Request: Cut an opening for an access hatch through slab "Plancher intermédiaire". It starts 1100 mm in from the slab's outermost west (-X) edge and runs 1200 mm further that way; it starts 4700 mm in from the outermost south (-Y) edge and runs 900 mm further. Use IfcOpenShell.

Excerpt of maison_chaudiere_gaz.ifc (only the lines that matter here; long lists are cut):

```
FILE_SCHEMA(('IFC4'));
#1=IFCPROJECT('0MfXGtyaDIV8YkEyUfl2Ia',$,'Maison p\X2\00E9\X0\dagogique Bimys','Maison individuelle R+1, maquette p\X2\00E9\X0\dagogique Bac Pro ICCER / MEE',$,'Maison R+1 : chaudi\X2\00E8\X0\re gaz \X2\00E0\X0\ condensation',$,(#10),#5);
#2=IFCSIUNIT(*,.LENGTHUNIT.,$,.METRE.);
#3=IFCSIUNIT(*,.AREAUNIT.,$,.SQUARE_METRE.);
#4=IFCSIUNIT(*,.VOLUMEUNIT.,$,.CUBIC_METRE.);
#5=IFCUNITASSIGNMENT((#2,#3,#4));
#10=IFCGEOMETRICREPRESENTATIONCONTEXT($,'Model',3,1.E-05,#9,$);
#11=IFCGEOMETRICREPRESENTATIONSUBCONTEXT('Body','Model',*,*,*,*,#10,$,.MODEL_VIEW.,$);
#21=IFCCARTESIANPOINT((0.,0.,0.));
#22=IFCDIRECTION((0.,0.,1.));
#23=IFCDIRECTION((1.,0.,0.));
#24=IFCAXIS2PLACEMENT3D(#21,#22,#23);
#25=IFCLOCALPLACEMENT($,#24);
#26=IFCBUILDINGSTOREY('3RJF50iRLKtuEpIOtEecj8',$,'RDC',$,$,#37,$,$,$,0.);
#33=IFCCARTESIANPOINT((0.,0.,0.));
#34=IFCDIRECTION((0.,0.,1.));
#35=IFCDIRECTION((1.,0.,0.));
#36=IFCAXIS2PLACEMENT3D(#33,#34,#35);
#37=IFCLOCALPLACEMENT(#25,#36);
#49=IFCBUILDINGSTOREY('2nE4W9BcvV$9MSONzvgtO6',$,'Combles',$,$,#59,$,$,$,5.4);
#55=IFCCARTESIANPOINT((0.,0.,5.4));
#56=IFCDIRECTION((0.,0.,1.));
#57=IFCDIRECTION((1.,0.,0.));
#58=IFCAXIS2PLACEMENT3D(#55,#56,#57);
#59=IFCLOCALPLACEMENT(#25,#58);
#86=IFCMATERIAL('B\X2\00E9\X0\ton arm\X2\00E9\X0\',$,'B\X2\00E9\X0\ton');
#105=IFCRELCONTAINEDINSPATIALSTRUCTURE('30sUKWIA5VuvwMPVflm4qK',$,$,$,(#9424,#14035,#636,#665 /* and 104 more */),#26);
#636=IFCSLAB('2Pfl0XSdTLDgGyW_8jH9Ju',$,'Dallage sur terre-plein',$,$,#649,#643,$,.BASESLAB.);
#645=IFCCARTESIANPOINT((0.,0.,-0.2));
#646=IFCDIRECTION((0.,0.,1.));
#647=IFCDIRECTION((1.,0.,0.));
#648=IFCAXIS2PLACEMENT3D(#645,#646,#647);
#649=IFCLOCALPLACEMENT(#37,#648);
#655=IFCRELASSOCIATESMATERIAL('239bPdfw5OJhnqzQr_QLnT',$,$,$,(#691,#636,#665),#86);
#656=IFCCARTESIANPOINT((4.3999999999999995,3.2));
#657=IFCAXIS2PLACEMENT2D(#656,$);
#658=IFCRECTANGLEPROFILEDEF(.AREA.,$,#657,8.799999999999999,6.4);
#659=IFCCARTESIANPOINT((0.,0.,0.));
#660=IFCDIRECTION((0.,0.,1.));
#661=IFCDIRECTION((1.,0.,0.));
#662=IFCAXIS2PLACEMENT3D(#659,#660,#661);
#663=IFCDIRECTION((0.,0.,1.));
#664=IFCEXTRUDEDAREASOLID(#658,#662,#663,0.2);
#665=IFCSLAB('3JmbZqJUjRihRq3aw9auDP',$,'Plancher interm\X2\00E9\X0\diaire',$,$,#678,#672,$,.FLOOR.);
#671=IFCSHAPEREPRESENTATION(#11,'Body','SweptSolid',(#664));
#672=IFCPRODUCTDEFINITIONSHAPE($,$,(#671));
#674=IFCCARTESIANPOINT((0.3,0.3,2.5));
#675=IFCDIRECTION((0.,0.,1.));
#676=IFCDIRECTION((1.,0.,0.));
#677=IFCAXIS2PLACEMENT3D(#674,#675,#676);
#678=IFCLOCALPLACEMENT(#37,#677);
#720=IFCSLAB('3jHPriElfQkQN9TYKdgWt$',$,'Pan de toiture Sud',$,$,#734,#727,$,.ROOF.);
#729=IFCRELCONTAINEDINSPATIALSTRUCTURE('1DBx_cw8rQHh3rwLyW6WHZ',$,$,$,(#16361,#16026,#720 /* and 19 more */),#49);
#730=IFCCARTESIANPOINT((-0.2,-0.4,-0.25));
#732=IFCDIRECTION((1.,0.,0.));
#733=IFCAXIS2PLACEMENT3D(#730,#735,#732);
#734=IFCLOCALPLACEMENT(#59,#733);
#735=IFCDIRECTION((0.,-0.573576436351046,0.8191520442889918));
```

```python
import numpy as np
import ifcopenshell
import ifcopenshell.api.feature
import ifcopenshell.api.geometry
import ifcopenshell.api.root
import ifcopenshell.geom
import ifcopenshell.util.placement
import ifcopenshell.util.representation
import ifcopenshell.util.shape
import ifcopenshell.util.unit

model = ifcopenshell.open("maison_chaudiere_gaz.ifc")
unit_scale = ifcopenshell.util.unit.calculate_unit_scale(model)
settings = ifcopenshell.geom.settings()


def volume(element):
    """Net volume in cubic metres, openings subtracted."""
    shape = ifcopenshell.geom.create_shape(settings, element)
    return ifcopenshell.util.shape.get_volume(shape.geometry)


slab = model.by_guid("3JmbZqJUjRihRq3aw9auDP")
before = volume(slab)

# Extent in the slab's own axes, in metres. The edges named are its -X and -Y sides.
slab_shape = ifcopenshell.geom.create_shape(settings, slab)
vertices = ifcopenshell.util.shape.get_vertices(slab_shape.geometry)
x_min, y_min, bottom = vertices.min(axis=0)
top = vertices[:, 2].max()

opening = ifcopenshell.api.root.create_entity(model, ifc_class="IfcOpeningElement", name="Access hatch opening", predefined_type="OPENING")
context = ifcopenshell.util.representation.get_context(model, "Model", "Body", "MODEL_VIEW")
width, depth = 1.2, 0.9
outline = [(0.0, 0.0), (width, 0.0), (width, depth), (0.0, depth), (0.0, 0.0)]
# Overshoot both faces by 50 mm so the cut is clean.
shape = ifcopenshell.api.geometry.add_slab_representation(
    model, context=context, depth=top - bottom + 0.1, polyline=outline
)
ifcopenshell.api.geometry.assign_representation(model, product=opening, representation=shape)

matrix = ifcopenshell.util.placement.get_local_placement(slab.ObjectPlacement)
matrix[:, 3] = matrix @ np.append(np.array([x_min + 1.1, y_min + 4.7, bottom - 0.05]) / unit_scale, 1.0)
ifcopenshell.api.geometry.edit_object_placement(model, product=opening, matrix=matrix, is_si=False)
ifcopenshell.api.feature.add_feature(model, feature=opening, element=slab)

after = volume(slab)

print(f"slab volume {before:.3f} -> {after:.3f} m3")

model.write("maison_chaudiere_gaz_v2.ifc")
```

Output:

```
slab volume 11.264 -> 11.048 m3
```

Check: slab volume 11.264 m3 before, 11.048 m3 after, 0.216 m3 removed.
